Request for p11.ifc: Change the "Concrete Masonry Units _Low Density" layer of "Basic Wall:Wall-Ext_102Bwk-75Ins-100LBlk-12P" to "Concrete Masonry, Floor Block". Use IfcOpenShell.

First a look at what the model holds.

```python
import ifcopenshell
import ifcopenshell.util.element

model = ifcopenshell.open("p11.ifc")
print(model.schema)
for layer_set in model.by_type("IfcMaterialLayerSet"):
    if layer_set.LayerSetName == "Basic Wall:Wall-Ext_102Bwk-75Ins-100LBlk-12P":
        for layer in layer_set.MaterialLayers:
            print(layer.id(), layer.Material and layer.Material.Name, layer.LayerThickness, sep=" | ")
        print(len(ifcopenshell.util.element.get_elements_by_material(model, layer_set)), "elements and types use it")
print(sorted(m.Name for m in model.by_type("IfcMaterial") if m.Name)[:60])
```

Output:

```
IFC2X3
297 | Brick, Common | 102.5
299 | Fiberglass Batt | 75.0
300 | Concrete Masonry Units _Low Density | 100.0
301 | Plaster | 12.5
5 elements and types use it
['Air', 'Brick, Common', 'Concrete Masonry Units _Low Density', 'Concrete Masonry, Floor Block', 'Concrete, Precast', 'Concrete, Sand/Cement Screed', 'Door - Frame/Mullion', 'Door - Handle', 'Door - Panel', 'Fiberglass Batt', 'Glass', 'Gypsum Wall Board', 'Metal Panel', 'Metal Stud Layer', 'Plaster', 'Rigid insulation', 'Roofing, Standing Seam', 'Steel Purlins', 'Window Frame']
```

```python
import ifcopenshell
import ifcopenshell.api.material

model = ifcopenshell.open("p11.ifc")

layer_set = next(s for s in model.by_type("IfcMaterialLayerSet") if s.LayerSetName == "Basic Wall:Wall-Ext_102Bwk-75Ins-100LBlk-12P")
layer = next(l for l in layer_set.MaterialLayers if l.Material and l.Material.Name == "Concrete Masonry Units _Low Density")
material = next(m for m in model.by_type("IfcMaterial") if m.Name == "Concrete Masonry, Floor Block")

# Point this one layer at the other material; renaming the old one would change it everywhere.
ifcopenshell.api.material.edit_layer(model, layer=layer, attributes={}, material=material)

print([l.Material.Name if l.Material else None for l in layer_set.MaterialLayers])

model.write("p11_v2.ifc")
```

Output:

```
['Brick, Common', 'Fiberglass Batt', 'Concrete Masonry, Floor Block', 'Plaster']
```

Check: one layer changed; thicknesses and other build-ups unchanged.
